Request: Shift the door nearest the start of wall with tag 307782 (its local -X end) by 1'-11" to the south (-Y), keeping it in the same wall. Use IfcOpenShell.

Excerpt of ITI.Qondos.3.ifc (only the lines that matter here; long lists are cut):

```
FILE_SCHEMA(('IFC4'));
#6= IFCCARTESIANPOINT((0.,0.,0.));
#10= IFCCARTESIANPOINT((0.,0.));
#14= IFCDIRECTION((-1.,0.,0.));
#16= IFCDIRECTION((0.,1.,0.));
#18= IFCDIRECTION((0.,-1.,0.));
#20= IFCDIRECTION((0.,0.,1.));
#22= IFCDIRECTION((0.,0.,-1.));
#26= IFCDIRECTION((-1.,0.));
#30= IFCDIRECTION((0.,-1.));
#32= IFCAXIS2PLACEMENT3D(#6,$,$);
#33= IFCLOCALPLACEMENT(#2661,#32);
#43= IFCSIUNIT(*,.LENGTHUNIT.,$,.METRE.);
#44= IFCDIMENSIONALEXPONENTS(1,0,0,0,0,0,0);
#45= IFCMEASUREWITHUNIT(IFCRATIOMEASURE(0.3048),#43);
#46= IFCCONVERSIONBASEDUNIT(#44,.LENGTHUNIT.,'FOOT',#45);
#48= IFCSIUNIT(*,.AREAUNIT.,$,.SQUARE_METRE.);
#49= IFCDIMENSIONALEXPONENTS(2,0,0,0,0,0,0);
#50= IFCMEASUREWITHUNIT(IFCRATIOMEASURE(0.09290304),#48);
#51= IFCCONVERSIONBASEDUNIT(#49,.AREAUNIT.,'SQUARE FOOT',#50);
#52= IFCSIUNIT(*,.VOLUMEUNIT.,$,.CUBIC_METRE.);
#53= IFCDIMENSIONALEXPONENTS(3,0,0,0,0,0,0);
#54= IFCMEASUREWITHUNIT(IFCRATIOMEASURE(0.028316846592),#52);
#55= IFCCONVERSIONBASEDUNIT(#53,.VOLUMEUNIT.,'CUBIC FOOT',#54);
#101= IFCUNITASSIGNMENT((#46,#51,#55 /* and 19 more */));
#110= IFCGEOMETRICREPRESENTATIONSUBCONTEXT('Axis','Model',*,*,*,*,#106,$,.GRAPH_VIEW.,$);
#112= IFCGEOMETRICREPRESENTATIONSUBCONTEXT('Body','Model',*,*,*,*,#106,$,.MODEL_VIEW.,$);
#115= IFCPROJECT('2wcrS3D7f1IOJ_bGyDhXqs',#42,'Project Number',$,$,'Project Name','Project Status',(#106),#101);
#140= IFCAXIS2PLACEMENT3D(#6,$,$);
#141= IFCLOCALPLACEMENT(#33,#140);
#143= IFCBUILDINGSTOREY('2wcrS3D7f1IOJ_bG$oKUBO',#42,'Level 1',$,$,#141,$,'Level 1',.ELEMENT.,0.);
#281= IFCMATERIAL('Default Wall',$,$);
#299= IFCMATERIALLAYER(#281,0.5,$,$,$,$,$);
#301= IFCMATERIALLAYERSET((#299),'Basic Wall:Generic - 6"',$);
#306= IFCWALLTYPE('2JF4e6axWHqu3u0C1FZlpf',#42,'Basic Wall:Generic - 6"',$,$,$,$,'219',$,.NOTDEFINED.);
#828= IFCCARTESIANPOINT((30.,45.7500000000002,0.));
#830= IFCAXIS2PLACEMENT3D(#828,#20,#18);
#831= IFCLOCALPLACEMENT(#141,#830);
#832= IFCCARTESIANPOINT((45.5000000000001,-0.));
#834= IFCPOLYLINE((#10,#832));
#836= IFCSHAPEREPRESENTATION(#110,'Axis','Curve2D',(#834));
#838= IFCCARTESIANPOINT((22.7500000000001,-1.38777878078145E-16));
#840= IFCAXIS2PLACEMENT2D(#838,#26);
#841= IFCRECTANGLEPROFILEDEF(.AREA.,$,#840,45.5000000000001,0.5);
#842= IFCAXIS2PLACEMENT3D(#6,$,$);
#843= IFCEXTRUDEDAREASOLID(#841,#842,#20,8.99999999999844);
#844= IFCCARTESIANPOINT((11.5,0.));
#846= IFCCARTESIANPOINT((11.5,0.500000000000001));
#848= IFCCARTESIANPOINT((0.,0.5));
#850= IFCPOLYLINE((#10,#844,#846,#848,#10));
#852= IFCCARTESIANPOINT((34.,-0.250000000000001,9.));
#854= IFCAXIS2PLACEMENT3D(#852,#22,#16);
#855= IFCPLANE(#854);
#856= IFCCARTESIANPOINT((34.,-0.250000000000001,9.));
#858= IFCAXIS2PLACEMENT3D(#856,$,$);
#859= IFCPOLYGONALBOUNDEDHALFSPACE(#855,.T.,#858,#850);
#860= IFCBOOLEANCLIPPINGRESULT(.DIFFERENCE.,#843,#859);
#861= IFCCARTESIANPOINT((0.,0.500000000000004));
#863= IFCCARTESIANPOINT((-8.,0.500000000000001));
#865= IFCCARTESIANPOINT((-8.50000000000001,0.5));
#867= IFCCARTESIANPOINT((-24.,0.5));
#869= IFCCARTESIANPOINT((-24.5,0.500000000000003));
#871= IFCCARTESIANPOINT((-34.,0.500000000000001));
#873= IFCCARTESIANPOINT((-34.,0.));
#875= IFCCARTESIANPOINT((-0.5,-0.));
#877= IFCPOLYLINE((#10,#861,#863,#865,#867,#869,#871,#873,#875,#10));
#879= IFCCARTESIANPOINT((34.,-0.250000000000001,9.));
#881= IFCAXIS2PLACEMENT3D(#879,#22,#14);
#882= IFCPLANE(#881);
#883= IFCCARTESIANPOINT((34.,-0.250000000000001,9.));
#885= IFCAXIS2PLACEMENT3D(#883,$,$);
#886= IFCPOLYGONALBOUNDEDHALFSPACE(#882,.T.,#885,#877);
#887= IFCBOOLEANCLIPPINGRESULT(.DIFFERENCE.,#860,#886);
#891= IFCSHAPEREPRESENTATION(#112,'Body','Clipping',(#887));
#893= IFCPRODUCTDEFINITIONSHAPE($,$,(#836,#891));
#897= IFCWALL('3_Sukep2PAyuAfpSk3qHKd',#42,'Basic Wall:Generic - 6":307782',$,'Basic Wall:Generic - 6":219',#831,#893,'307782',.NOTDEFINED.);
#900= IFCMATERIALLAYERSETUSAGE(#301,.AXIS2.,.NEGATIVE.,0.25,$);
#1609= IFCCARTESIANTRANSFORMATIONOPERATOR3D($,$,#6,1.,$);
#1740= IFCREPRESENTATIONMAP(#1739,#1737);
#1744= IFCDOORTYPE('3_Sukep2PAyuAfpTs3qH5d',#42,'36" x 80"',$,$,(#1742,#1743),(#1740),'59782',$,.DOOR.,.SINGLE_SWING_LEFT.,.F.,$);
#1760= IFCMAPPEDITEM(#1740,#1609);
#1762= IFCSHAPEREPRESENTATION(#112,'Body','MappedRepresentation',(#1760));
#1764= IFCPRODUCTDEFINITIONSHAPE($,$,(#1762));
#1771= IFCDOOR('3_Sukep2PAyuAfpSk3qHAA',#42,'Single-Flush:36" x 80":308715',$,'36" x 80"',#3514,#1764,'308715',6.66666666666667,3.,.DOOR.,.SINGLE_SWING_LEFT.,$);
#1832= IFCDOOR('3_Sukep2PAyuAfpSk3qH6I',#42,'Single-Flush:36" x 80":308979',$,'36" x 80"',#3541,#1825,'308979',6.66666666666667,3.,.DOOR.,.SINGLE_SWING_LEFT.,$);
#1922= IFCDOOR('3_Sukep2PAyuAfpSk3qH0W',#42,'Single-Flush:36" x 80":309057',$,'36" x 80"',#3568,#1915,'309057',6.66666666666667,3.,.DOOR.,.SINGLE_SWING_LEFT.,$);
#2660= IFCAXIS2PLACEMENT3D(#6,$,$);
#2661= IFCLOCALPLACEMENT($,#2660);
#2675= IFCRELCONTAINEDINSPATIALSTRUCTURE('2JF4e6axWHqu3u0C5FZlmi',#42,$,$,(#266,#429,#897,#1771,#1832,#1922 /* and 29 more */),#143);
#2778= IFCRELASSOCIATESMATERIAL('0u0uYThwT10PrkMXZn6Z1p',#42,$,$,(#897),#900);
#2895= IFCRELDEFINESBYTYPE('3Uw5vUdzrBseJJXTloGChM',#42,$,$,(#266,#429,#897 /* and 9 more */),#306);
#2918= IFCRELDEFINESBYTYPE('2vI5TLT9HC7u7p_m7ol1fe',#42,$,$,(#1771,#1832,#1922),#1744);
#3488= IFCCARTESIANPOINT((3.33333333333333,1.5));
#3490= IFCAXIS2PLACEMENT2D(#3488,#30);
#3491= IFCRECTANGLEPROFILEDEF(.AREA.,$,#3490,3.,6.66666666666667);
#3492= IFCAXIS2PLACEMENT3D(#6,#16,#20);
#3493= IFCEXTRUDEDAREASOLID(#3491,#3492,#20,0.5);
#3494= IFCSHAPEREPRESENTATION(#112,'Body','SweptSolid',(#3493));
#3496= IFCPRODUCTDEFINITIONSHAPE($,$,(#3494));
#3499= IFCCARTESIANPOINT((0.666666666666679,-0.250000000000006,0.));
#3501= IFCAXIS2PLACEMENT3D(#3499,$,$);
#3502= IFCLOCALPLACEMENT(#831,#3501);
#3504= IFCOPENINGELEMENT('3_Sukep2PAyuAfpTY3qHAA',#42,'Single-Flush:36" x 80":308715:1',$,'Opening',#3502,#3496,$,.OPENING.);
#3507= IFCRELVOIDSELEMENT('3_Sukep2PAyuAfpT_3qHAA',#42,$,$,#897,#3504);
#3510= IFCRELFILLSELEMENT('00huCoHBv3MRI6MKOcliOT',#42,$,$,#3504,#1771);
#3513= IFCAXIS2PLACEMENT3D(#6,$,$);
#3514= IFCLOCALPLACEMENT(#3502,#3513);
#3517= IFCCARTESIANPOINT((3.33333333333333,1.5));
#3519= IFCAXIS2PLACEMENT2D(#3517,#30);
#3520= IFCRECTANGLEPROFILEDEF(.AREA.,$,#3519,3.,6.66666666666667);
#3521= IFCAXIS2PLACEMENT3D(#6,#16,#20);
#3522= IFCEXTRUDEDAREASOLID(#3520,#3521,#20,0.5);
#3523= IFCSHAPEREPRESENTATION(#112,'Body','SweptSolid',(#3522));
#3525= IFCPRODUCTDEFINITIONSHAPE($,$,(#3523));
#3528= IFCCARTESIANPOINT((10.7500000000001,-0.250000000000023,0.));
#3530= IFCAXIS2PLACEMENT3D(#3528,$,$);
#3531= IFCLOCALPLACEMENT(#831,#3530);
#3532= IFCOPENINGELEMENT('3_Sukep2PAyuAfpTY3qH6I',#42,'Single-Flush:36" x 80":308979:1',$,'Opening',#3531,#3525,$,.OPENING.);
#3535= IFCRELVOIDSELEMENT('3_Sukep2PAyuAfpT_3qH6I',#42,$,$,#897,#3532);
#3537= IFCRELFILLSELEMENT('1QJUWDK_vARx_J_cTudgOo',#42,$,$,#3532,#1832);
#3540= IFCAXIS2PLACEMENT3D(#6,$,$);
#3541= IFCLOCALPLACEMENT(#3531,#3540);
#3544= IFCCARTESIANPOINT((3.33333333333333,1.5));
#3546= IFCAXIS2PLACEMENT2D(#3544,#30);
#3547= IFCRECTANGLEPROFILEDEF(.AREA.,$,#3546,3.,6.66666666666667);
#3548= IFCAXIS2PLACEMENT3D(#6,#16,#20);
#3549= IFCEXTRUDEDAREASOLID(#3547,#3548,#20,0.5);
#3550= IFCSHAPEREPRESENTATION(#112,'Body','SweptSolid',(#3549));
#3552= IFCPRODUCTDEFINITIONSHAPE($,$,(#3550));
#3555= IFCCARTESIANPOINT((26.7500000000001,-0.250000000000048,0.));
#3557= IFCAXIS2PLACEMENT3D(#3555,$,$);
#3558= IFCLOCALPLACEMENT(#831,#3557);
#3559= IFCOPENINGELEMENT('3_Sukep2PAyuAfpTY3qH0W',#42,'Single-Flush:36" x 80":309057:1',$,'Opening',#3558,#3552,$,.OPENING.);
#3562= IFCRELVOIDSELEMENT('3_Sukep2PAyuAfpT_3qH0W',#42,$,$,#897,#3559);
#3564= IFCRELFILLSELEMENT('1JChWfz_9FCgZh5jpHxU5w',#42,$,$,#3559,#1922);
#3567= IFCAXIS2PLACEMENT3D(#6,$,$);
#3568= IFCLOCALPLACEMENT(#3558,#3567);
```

```python
import ifcopenshell
import ifcopenshell.api.geometry
import ifcopenshell.util.placement
import ifcopenshell.util.unit

model = ifcopenshell.open("ITI.Qondos.3.ifc")
unit_scale = ifcopenshell.util.unit.calculate_unit_scale(model)

door = model.by_guid("3_Sukep2PAyuAfpSk3qHAA")
opening = door.FillsVoids[0].RelatingOpeningElement
wall = opening.VoidsElements[0].RelatingBuildingElement

wall_matrix = ifcopenshell.util.placement.get_local_placement(wall.ObjectPlacement)
shift = wall_matrix[:3, 0] * 23 * 0.0254 / unit_scale
before = ifcopenshell.util.placement.get_local_placement(door.ObjectPlacement)[:3, 3].copy()

# The door is placed relative to its opening, so it follows when the opening moves.
matrix = ifcopenshell.util.placement.get_local_placement(opening.ObjectPlacement)
matrix[:3, 3] += shift
ifcopenshell.api.geometry.edit_object_placement(
    model, product=opening, matrix=matrix, is_si=False, should_transform_children=True
)

after = ifcopenshell.util.placement.get_local_placement(door.ObjectPlacement)[:3, 3]
print("door moved by", (after - before).round(3) + 0.0)

model.write("ITI.Qondos.3_v2.ifc")
```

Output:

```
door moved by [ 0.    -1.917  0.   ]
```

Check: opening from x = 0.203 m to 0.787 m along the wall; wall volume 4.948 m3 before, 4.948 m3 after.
